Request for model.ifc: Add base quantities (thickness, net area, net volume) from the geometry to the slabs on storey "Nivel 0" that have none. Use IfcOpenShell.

First a look at what the model holds.

```python
import ifcopenshell
import ifcopenshell.util.element
import ifcopenshell.util.unit

model = ifcopenshell.open("model.ifc")
print(model.schema)
for unit_type in ("LENGTHUNIT", "AREAUNIT", "VOLUMEUNIT"):
    print(unit_type, ifcopenshell.util.unit.calculate_unit_scale(model, unit_type))
storey = next(s for s in model.by_type("IfcBuildingStorey") if s.Name == "Nivel 0")
slabs = [e for e in ifcopenshell.util.element.get_decomposition(storey) if e.is_a("IfcSlab")]
for e in sorted(slabs, key=lambda e: e.id()):
    print(e.id(), e.is_a(), e.Name, list(ifcopenshell.util.element.get_psets(e, qtos_only=True)), sep=" | ")
```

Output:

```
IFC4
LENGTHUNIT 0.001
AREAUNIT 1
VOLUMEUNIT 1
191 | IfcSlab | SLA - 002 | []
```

```python
import ifcopenshell
import ifcopenshell.api.pset
import ifcopenshell.geom
import ifcopenshell.util.element
import ifcopenshell.util.shape
import ifcopenshell.util.unit

model = ifcopenshell.open("model.ifc")
unit_scale = ifcopenshell.util.unit.calculate_unit_scale(model)
area_scale = ifcopenshell.util.unit.calculate_unit_scale(model, "AREAUNIT")
volume_scale = ifcopenshell.util.unit.calculate_unit_scale(model, "VOLUMEUNIT")
settings = ifcopenshell.geom.settings()

storey = next(s for s in model.by_type("IfcBuildingStorey") if s.Name == "Nivel 0")
slabs = [e for e in ifcopenshell.util.element.get_decomposition(storey) if e.is_a("IfcSlab")]

for e in sorted(slabs, key=lambda e: e.id()):
    if ifcopenshell.util.element.get_psets(e, qtos_only=True, should_inherit=False):
        continue
    # Geometry comes back in metres, in the element's own axes.
    shape = ifcopenshell.geom.create_shape(settings, e)
    values = {
        "Width": ifcopenshell.util.shape.get_z(shape.geometry) / unit_scale,
        "NetArea": ifcopenshell.util.shape.get_footprint_area(shape.geometry) / area_scale,
        "NetVolume": ifcopenshell.util.shape.get_volume(shape.geometry) / volume_scale,
    }
    qto = ifcopenshell.api.pset.add_qto(model, product=e, name="Qto_SlabBaseQuantities")
    ifcopenshell.api.pset.edit_qto(model, qto=qto, properties=values)
    print(e.id(), {k: round(v, 3) for k, v in values.items()})

model.write("model_rev.ifc")
```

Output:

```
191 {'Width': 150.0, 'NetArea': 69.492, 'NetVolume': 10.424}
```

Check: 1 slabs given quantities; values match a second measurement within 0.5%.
